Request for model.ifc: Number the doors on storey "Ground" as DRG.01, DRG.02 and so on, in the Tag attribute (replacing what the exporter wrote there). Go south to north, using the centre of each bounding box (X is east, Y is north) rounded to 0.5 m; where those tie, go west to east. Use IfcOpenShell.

First a look at what the model holds.

```python
import ifcopenshell
import ifcopenshell.util.element
import ifcopenshell.util.placement

model = ifcopenshell.open("model.ifc")
print(model.schema)
storey = next(s for s in model.by_type("IfcBuildingStorey") if s.Name == "Ground")
doors = [e for e in ifcopenshell.util.element.get_decomposition(storey) if e.is_a("IfcDoor")]
for e in sorted(doors, key=lambda e: e.id()):
    origin = ifcopenshell.util.placement.get_local_placement(e.ObjectPlacement)[:3, 3]
    print(e.id(), e.Tag, e.Name, origin.round(2) + 0.0, sep=" | ")
```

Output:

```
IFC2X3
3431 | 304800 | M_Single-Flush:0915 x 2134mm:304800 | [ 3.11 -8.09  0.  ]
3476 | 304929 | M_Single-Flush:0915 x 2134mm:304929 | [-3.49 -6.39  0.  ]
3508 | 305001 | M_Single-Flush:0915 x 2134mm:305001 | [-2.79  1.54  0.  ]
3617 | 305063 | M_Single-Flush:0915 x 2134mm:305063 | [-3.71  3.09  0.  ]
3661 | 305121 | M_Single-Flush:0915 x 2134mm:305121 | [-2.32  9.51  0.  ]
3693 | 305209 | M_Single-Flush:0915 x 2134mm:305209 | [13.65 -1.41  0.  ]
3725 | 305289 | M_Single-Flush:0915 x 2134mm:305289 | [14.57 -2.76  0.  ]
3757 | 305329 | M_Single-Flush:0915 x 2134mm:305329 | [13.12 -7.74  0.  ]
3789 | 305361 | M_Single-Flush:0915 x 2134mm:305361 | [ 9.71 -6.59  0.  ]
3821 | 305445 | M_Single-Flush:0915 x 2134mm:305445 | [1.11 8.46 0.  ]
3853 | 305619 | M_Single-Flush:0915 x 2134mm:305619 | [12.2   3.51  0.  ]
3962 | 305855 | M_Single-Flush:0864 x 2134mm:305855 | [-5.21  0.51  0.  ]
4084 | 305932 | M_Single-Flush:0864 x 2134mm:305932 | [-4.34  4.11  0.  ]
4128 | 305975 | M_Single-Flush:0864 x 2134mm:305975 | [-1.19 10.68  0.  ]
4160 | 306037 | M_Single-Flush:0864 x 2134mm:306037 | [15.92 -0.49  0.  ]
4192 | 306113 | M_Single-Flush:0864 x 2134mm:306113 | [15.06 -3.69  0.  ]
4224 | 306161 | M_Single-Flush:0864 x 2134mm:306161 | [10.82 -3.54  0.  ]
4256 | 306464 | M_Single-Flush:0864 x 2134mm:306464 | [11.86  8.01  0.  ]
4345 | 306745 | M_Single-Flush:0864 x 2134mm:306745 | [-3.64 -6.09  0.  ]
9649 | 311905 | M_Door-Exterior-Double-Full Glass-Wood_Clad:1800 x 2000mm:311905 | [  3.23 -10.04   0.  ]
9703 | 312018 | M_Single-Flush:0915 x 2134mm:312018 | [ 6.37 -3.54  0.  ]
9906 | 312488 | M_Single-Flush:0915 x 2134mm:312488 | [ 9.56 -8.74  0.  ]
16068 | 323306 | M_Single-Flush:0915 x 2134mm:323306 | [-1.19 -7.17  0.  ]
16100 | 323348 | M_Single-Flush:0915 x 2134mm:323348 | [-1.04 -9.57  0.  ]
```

```python
import ifcopenshell
import ifcopenshell.geom
import ifcopenshell.util.element
import ifcopenshell.util.shape

model = ifcopenshell.open("model.ifc")
settings = ifcopenshell.geom.settings()
settings.set("use-world-coords", True)


def centre(element):
    shape = ifcopenshell.geom.create_shape(settings, element)
    return ifcopenshell.util.shape.get_bbox_centroid(shape.geometry)


storey = next(s for s in model.by_type("IfcBuildingStorey") if s.Name == "Ground")
doors = [e for e in ifcopenshell.util.element.get_decomposition(storey) if e.is_a("IfcDoor")]

# Insertion points can sit at a corner or the storey origin, so sort by the geometry (in metres).
centres = {e: centre(e) for e in doors}
doors.sort(key=lambda e: (round(centres[e][1] / 0.5), centres[e][0]))

for i, e in enumerate(doors, start=1):
    number = f"DRG.{i:02d}"
    e.Tag = number
    print(e.id(), number)

model.write("model_edited.ifc")
```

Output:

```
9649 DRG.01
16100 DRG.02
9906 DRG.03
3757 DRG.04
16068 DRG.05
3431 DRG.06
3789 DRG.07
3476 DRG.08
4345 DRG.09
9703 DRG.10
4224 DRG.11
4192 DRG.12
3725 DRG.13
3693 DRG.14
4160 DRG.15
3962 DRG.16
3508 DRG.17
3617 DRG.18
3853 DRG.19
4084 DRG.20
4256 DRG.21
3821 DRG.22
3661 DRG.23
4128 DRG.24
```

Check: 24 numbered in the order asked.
